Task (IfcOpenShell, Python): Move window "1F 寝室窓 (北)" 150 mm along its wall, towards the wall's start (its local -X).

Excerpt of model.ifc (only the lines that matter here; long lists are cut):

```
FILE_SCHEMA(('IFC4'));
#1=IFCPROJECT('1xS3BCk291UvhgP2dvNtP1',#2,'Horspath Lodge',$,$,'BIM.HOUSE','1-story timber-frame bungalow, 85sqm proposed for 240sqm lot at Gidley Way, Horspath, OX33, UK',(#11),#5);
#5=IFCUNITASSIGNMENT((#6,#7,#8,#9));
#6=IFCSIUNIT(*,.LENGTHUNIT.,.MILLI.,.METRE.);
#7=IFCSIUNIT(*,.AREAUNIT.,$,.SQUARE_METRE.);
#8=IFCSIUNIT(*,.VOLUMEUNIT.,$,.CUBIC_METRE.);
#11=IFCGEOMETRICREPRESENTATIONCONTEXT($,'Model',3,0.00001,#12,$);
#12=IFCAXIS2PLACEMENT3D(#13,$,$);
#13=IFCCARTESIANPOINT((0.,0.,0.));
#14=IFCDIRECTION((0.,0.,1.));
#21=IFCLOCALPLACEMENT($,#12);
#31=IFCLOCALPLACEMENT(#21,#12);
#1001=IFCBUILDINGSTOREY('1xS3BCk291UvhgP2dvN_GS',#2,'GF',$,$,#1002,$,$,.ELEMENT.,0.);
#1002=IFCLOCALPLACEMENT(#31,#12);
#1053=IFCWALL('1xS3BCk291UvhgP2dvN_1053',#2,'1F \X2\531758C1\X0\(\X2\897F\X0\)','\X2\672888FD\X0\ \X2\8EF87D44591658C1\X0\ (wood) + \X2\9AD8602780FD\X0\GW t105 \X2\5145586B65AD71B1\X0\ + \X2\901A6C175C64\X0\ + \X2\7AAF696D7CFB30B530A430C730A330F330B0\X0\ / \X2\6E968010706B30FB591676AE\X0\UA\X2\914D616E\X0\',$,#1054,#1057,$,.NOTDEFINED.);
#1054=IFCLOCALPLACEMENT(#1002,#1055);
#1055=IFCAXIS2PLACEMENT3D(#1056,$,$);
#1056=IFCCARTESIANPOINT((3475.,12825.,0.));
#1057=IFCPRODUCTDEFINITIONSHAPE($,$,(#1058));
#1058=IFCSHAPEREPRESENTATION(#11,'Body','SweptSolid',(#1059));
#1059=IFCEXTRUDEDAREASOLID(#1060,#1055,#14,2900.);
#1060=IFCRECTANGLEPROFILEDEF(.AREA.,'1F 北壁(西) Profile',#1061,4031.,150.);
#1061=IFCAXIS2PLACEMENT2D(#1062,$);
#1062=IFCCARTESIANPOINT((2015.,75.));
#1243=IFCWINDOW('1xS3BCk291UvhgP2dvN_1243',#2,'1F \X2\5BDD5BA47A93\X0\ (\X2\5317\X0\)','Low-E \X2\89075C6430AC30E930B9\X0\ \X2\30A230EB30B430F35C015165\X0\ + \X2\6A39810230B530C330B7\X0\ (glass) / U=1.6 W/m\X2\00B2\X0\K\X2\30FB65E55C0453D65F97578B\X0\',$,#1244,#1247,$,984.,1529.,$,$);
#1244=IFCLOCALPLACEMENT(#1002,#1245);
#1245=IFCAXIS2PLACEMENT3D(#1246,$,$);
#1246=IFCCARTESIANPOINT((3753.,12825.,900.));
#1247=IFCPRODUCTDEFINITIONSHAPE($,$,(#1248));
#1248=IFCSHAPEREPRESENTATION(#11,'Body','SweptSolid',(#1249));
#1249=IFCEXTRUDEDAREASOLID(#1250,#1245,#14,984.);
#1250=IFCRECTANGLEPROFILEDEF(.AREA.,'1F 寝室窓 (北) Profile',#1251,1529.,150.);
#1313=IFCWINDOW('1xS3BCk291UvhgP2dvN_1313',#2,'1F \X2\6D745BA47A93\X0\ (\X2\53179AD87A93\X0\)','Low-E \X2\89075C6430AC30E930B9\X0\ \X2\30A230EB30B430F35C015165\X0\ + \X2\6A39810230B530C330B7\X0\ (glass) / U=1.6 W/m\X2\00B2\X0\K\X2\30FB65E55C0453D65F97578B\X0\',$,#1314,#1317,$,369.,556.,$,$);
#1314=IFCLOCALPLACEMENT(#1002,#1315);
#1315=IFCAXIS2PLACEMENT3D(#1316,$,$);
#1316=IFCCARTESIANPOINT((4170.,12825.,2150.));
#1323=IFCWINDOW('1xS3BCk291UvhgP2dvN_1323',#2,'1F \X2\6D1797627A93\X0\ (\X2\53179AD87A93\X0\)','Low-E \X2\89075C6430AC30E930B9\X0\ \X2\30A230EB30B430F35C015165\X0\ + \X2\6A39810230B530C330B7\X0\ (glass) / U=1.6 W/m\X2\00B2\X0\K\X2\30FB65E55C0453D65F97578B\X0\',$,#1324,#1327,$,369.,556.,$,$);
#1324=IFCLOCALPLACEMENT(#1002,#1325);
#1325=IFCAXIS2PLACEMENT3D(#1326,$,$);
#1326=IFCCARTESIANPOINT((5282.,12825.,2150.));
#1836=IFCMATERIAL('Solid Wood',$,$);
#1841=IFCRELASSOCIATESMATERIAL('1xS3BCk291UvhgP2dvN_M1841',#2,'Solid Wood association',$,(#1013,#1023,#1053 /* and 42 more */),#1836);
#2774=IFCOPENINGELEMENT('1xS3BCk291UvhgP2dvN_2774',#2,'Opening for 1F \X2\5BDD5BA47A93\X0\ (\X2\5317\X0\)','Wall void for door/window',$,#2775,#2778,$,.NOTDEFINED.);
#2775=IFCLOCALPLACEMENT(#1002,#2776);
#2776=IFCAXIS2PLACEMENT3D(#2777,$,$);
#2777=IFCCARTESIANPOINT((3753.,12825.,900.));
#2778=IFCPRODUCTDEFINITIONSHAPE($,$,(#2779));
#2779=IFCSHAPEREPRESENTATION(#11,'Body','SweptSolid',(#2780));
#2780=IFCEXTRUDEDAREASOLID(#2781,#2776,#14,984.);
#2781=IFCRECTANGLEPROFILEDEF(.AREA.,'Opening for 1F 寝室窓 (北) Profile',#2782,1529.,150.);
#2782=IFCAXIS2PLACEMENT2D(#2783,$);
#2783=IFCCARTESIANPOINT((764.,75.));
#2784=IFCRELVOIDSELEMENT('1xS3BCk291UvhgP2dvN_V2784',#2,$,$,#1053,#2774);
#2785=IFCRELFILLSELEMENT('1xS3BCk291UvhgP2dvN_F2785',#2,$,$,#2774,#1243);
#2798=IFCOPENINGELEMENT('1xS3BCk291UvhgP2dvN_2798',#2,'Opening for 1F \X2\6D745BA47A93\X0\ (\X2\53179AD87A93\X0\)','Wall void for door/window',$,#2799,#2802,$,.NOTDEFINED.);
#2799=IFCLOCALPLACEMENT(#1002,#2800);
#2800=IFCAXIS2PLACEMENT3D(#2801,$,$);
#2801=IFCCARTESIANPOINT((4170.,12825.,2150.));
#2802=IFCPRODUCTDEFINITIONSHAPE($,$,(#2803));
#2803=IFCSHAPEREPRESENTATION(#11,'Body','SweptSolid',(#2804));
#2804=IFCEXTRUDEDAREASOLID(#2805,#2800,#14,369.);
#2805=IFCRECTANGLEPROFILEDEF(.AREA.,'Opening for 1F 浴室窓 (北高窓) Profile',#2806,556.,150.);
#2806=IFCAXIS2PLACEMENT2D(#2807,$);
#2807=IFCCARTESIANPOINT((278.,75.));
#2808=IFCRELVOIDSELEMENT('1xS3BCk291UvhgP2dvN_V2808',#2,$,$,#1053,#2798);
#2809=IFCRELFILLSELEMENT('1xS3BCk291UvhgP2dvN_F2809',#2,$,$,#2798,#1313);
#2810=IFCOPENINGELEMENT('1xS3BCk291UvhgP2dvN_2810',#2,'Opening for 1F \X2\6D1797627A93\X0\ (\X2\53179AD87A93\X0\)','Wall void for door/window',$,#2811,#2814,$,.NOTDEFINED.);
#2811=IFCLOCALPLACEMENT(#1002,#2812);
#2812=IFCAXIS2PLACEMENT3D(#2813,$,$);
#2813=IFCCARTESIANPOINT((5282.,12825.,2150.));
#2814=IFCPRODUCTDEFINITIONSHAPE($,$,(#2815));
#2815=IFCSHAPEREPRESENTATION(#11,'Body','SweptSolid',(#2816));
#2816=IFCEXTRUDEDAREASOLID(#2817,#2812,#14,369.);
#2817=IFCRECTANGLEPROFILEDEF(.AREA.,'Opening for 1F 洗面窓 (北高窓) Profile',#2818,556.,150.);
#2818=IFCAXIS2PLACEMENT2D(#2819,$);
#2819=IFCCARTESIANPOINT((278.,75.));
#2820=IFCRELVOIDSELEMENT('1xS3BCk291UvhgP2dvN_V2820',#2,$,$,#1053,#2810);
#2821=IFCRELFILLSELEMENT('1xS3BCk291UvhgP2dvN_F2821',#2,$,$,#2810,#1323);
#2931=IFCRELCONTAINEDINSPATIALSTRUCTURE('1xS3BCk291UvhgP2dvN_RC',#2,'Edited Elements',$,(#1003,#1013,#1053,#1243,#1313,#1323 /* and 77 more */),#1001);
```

```python
import ifcopenshell
import ifcopenshell.api.geometry
import ifcopenshell.util.placement
import ifcopenshell.util.unit

model = ifcopenshell.open("model.ifc")
unit_scale = ifcopenshell.util.unit.calculate_unit_scale(model)

window = model.by_id(1243)
opening = window.FillsVoids[0].RelatingOpeningElement
wall = opening.VoidsElements[0].RelatingBuildingElement

wall_matrix = ifcopenshell.util.placement.get_local_placement(wall.ObjectPlacement)
shift = wall_matrix[:3, 0] * -0.15 / unit_scale
before = ifcopenshell.util.placement.get_local_placement(window.ObjectPlacement)[:3, 3].copy()

# The window is not placed relative to its opening, so move both.
for product in (opening, window):
    matrix = ifcopenshell.util.placement.get_local_placement(product.ObjectPlacement)
    matrix[:3, 3] += shift
    ifcopenshell.api.geometry.edit_object_placement(model, product=product, matrix=matrix, is_si=False)

after = ifcopenshell.util.placement.get_local_placement(window.ObjectPlacement)[:3, 3]
print("window moved by", (after - before).round(3) + 0.0)

model.write("model_rev.ifc")
```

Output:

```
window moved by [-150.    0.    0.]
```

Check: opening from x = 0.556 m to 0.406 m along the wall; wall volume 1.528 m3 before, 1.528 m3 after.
